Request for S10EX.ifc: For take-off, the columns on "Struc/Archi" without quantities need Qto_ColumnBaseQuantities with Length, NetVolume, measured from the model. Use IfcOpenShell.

First a look at what the model holds.

```python
import ifcopenshell
import ifcopenshell.util.element
import ifcopenshell.util.unit

model = ifcopenshell.open("S10EX.ifc")
print(model.schema)
for unit_type in ("LENGTHUNIT", "AREAUNIT", "VOLUMEUNIT"):
    print(unit_type, ifcopenshell.util.unit.calculate_unit_scale(model, unit_type))
storey = next(s for s in model.by_type("IfcBuildingStorey") if s.Name == "Struc/Archi")
columns = [e for e in ifcopenshell.util.element.get_decomposition(storey) if e.is_a("IfcColumn")]
for e in sorted(columns, key=lambda e: e.id()):
    print(e.id(), e.is_a(), e.Name, list(ifcopenshell.util.element.get_psets(e, qtos_only=True)), sep=" | ")
```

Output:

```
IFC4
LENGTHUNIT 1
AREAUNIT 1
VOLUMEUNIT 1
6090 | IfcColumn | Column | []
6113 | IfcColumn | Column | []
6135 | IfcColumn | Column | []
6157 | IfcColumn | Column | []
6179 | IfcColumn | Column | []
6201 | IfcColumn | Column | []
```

```python
import ifcopenshell
import ifcopenshell.api.pset
import ifcopenshell.geom
import ifcopenshell.util.element
import ifcopenshell.util.shape
import ifcopenshell.util.unit

model = ifcopenshell.open("S10EX.ifc")
unit_scale = ifcopenshell.util.unit.calculate_unit_scale(model)
volume_scale = ifcopenshell.util.unit.calculate_unit_scale(model, "VOLUMEUNIT")
settings = ifcopenshell.geom.settings()

storey = next(s for s in model.by_type("IfcBuildingStorey") if s.Name == "Struc/Archi")
columns = [e for e in ifcopenshell.util.element.get_decomposition(storey) if e.is_a("IfcColumn")]

for e in sorted(columns, key=lambda e: e.id()):
    if ifcopenshell.util.element.get_psets(e, qtos_only=True, should_inherit=False):
        continue
    # Geometry comes back in metres, in the element's own axes.
    shape = ifcopenshell.geom.create_shape(settings, e)
    values = {
        "Length": ifcopenshell.util.shape.get_z(shape.geometry) / unit_scale,
        "NetVolume": ifcopenshell.util.shape.get_volume(shape.geometry) / volume_scale,
    }
    qto = ifcopenshell.api.pset.add_qto(model, product=e, name="Qto_ColumnBaseQuantities")
    ifcopenshell.api.pset.edit_qto(model, qto=qto, properties=values)
    print(e.id(), {k: round(v, 3) for k, v in values.items()})

model.write("S10EX_v2.ifc")
```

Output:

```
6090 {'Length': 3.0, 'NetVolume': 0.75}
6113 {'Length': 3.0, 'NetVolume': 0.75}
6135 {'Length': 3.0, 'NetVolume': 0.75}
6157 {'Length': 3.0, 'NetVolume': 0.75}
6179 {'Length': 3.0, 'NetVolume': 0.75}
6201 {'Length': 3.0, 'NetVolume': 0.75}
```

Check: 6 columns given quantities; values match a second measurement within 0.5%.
